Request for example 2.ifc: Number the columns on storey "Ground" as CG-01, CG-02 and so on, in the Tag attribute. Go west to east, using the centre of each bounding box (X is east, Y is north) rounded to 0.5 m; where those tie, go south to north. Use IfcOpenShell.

First a look at what the model holds.

```python
import ifcopenshell
import ifcopenshell.util.element
import ifcopenshell.util.placement

model = ifcopenshell.open("example 2.ifc")
print(model.schema)
storey = next(s for s in model.by_type("IfcBuildingStorey") if s.Name == "Ground")
columns = [e for e in ifcopenshell.util.element.get_decomposition(storey) if e.is_a("IfcColumn")]
for e in sorted(columns, key=lambda e: e.id()):
    origin = ifcopenshell.util.placement.get_local_placement(e.ObjectPlacement)[:3, 3]
    print(e.id(), e.Tag, e.Name, origin.round(2) + 0.0, sep=" | ")
```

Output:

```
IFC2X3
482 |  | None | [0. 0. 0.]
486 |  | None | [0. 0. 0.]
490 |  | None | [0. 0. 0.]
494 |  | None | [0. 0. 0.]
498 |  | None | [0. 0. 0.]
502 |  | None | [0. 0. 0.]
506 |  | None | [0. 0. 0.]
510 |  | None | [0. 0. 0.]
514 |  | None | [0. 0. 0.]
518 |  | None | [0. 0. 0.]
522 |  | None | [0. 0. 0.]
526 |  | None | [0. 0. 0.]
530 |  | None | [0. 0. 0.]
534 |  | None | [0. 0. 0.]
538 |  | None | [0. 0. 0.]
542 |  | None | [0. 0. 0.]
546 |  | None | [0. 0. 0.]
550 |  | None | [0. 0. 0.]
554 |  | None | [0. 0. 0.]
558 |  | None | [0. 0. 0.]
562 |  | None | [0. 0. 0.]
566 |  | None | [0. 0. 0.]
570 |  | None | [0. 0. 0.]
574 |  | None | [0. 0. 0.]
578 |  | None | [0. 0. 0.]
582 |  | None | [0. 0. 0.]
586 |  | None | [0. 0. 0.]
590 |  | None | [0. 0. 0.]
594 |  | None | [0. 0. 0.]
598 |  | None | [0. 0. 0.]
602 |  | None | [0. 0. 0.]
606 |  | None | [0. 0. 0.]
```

```python
import ifcopenshell
import ifcopenshell.geom
import ifcopenshell.util.element
import ifcopenshell.util.shape

model = ifcopenshell.open("example 2.ifc")
settings = ifcopenshell.geom.settings()
settings.set("use-world-coords", True)


def centre(element):
    shape = ifcopenshell.geom.create_shape(settings, element)
    return ifcopenshell.util.shape.get_bbox_centroid(shape.geometry)


storey = next(s for s in model.by_type("IfcBuildingStorey") if s.Name == "Ground")
columns = [e for e in ifcopenshell.util.element.get_decomposition(storey) if e.is_a("IfcColumn")]

# Insertion points can sit at a corner or the storey origin, so sort by the geometry (in metres).
centres = {e: centre(e) for e in columns}
columns.sort(key=lambda e: (round(centres[e][0] / 0.5), centres[e][1]))

for i, e in enumerate(columns, start=1):
    number = f"CG-{i:02d}"
    e.Tag = number
    print(e.id(), number)

model.write("example 2-out.ifc")
```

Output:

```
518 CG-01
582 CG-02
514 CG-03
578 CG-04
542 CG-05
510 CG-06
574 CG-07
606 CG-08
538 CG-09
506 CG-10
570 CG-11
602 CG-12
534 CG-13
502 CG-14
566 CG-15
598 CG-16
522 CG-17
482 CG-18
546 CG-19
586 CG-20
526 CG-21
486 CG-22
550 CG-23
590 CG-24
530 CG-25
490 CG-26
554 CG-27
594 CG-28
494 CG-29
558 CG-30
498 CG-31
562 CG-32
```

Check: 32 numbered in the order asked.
